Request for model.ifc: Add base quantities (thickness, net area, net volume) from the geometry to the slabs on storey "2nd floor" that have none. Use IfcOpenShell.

First a look at what the model holds.

```python
import ifcopenshell
import ifcopenshell.util.element
import ifcopenshell.util.unit

model = ifcopenshell.open("model.ifc")
print(model.schema)
for unit_type in ("LENGTHUNIT", "AREAUNIT", "VOLUMEUNIT"):
    print(unit_type, ifcopenshell.util.unit.calculate_unit_scale(model, unit_type))
storey = next(s for s in model.by_type("IfcBuildingStorey") if s.Name == "2nd floor")
slabs = [e for e in ifcopenshell.util.element.get_decomposition(storey) if e.is_a("IfcSlab")]
for e in sorted(slabs, key=lambda e: e.id()):
    print(e.id(), e.is_a(), e.Name, list(ifcopenshell.util.element.get_psets(e, qtos_only=True)), sep=" | ")
```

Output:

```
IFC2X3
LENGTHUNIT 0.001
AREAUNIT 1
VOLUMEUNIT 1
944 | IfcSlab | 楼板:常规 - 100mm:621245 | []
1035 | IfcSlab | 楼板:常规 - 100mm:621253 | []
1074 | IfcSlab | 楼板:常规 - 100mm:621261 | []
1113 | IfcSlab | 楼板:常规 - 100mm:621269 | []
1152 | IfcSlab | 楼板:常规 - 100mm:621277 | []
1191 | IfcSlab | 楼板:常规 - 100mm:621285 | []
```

```python
import ifcopenshell
import ifcopenshell.api.pset
import ifcopenshell.geom
import ifcopenshell.util.element
import ifcopenshell.util.shape
import ifcopenshell.util.unit

model = ifcopenshell.open("model.ifc")
unit_scale = ifcopenshell.util.unit.calculate_unit_scale(model)
area_scale = ifcopenshell.util.unit.calculate_unit_scale(model, "AREAUNIT")
volume_scale = ifcopenshell.util.unit.calculate_unit_scale(model, "VOLUMEUNIT")
settings = ifcopenshell.geom.settings()

storey = next(s for s in model.by_type("IfcBuildingStorey") if s.Name == "2nd floor")
slabs = [e for e in ifcopenshell.util.element.get_decomposition(storey) if e.is_a("IfcSlab")]

for e in sorted(slabs, key=lambda e: e.id()):
    if ifcopenshell.util.element.get_psets(e, qtos_only=True, should_inherit=False):
        continue
    # Geometry comes back in metres, in the element's own axes.
    shape = ifcopenshell.geom.create_shape(settings, e)
    values = {
        "Width": ifcopenshell.util.shape.get_z(shape.geometry) / unit_scale,
        "NetArea": ifcopenshell.util.shape.get_footprint_area(shape.geometry) / area_scale,
        "NetVolume": ifcopenshell.util.shape.get_volume(shape.geometry) / volume_scale,
    }
    qto = ifcopenshell.api.pset.add_qto(model, product=e, name="BaseQuantities")
    ifcopenshell.api.pset.edit_qto(model, qto=qto, properties=values)
    print(e.id(), {k: round(v, 3) for k, v in values.items()})

model.write("model_v2.ifc")
```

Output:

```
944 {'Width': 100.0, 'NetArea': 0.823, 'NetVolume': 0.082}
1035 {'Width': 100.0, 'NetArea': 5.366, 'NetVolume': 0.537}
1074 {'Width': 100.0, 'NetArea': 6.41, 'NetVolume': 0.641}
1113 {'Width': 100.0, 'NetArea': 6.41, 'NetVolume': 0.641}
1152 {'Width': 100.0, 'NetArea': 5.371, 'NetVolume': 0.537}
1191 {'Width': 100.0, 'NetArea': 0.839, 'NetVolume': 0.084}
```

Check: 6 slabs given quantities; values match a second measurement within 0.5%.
